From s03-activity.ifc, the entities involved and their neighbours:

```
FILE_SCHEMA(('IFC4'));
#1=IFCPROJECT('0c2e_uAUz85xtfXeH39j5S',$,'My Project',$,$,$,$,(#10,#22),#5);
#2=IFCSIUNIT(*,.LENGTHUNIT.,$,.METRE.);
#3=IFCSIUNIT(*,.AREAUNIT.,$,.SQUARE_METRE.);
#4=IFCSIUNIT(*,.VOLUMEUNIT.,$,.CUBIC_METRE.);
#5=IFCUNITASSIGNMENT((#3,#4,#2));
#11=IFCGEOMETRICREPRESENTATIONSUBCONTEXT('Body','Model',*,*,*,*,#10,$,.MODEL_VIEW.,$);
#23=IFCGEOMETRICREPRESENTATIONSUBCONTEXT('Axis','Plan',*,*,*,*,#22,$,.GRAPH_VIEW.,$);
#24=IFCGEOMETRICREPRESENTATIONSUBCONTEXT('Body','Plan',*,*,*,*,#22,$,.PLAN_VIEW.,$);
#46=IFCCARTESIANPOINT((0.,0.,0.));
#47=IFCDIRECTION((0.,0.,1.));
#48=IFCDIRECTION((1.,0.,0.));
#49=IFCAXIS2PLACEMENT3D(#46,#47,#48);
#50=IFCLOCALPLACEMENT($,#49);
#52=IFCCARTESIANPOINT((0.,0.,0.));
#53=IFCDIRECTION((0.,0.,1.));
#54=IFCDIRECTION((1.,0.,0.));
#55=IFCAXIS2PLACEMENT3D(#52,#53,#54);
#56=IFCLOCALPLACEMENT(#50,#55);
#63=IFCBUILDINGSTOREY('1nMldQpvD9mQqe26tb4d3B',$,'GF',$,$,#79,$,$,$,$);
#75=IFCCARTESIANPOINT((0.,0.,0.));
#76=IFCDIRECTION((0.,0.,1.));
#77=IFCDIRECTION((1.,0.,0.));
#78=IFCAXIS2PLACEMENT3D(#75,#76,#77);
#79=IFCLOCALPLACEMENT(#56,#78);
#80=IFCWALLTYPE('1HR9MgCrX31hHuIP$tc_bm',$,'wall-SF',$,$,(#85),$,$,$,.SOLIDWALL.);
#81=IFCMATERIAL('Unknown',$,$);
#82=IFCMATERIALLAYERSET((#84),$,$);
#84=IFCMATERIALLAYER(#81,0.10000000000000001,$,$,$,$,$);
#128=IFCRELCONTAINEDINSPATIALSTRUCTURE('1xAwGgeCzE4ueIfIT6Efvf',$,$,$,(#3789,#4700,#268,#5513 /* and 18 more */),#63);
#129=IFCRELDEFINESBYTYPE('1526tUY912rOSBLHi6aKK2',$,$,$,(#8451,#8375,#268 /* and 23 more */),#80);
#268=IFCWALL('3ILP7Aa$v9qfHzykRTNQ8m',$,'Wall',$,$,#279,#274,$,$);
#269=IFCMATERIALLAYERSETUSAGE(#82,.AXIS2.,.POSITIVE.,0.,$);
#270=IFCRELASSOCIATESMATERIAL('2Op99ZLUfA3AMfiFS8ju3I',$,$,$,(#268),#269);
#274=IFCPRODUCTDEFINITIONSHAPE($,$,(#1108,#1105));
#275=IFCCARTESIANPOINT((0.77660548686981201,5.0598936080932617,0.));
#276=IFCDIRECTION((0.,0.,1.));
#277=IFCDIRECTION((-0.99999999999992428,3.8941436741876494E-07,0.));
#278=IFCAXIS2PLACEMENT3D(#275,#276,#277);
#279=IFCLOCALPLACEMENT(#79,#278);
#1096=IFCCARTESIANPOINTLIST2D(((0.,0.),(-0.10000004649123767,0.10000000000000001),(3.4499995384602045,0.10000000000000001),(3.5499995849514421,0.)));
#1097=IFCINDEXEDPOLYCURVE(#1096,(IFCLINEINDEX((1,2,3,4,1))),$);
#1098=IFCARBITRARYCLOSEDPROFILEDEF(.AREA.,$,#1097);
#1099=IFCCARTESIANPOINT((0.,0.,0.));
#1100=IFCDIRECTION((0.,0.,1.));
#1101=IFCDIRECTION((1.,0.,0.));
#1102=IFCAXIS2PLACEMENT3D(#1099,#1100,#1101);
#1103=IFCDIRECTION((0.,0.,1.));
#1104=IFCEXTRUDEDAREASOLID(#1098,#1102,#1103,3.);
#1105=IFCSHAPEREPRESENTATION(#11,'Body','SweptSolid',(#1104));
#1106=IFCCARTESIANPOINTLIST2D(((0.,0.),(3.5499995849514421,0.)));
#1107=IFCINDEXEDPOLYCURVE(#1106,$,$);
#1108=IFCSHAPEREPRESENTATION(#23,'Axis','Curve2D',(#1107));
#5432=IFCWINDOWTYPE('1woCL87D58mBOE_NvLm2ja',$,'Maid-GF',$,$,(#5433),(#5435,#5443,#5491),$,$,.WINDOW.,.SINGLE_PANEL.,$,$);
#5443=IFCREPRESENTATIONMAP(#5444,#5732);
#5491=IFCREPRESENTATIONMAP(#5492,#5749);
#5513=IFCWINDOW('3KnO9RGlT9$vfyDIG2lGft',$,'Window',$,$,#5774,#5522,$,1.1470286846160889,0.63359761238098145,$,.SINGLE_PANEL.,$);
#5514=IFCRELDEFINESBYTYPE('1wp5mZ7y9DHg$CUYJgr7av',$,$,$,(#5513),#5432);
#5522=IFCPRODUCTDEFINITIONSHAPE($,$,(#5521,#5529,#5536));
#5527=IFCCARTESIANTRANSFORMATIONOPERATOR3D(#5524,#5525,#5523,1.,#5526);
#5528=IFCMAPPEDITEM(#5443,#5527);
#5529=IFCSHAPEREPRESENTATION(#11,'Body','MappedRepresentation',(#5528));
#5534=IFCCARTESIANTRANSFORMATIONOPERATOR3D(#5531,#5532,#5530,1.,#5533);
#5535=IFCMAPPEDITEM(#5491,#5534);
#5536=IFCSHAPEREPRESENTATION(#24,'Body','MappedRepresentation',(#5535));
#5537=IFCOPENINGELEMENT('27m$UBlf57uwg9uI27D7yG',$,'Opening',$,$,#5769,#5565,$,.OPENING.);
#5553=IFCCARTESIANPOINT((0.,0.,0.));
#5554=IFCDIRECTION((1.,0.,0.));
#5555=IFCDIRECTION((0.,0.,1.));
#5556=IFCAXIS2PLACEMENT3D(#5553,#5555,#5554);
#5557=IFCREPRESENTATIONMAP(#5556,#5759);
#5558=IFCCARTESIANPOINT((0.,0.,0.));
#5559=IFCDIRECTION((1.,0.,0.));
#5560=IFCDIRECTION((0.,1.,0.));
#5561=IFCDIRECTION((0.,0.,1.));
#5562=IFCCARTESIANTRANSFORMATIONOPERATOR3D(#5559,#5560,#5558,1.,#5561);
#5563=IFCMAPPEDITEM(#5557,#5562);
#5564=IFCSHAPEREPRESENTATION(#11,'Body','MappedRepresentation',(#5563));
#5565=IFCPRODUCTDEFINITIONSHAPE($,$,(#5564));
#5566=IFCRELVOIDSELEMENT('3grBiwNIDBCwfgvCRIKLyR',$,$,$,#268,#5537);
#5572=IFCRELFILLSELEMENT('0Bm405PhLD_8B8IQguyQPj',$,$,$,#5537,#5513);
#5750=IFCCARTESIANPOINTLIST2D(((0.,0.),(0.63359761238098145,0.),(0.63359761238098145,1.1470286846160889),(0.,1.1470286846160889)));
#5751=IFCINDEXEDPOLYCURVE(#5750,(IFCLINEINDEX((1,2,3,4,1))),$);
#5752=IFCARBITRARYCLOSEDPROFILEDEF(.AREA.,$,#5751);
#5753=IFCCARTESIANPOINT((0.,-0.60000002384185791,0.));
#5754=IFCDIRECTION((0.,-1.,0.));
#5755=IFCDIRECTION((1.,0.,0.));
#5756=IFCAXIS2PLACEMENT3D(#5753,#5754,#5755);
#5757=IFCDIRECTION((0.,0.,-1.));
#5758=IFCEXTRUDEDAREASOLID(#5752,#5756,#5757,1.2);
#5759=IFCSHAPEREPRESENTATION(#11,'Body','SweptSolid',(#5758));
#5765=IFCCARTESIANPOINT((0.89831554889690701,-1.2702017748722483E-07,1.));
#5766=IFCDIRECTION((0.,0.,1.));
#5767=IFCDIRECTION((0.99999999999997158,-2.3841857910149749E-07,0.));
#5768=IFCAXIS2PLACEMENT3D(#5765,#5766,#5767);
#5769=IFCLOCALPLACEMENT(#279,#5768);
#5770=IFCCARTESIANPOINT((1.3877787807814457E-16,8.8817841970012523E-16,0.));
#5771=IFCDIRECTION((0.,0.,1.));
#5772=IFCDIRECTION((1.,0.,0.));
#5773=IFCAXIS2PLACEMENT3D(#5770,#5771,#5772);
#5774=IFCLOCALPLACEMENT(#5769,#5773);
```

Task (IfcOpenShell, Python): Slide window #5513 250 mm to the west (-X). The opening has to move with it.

```python
import ifcopenshell
import ifcopenshell.api.geometry
import ifcopenshell.util.placement
import ifcopenshell.util.unit

model = ifcopenshell.open("s03-activity.ifc")
unit_scale = ifcopenshell.util.unit.calculate_unit_scale(model)

window = model.by_guid("3KnO9RGlT9$vfyDIG2lGft")
opening = window.FillsVoids[0].RelatingOpeningElement
wall = opening.VoidsElements[0].RelatingBuildingElement

wall_matrix = ifcopenshell.util.placement.get_local_placement(wall.ObjectPlacement)
shift = wall_matrix[:3, 0] * 0.25 / unit_scale
before = ifcopenshell.util.placement.get_local_placement(window.ObjectPlacement)[:3, 3].copy()

# The window is placed relative to its opening, so it follows when the opening moves.
matrix = ifcopenshell.util.placement.get_local_placement(opening.ObjectPlacement)
matrix[:3, 3] += shift
ifcopenshell.api.geometry.edit_object_placement(
    model, product=opening, matrix=matrix, is_si=False, should_transform_children=True
)

after = ifcopenshell.util.placement.get_local_placement(window.ObjectPlacement)[:3, 3]
print("window moved by", (after - before).round(3) + 0.0)

model.write("s03-activity_updated.ifc")
```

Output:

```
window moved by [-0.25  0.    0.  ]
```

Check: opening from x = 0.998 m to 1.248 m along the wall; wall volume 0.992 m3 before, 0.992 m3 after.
